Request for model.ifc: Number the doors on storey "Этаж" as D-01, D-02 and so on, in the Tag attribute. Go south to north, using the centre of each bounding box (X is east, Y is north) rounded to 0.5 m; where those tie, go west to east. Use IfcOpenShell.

First a look at what the model holds.

```python
import ifcopenshell
import ifcopenshell.util.element
import ifcopenshell.util.placement

model = ifcopenshell.open("model.ifc")
print(model.schema)
storey = next(s for s in model.by_type("IfcBuildingStorey") if s.Name == "Этаж")
doors = [e for e in ifcopenshell.util.element.get_decomposition(storey) if e.is_a("IfcDoor")]
for e in sorted(doors, key=lambda e: e.id()):
    origin = ifcopenshell.util.placement.get_local_placement(e.ObjectPlacement)[:3, 3]
    print(e.id(), e.Tag, e.Name, origin.round(2) + 0.0, sep=" | ")
```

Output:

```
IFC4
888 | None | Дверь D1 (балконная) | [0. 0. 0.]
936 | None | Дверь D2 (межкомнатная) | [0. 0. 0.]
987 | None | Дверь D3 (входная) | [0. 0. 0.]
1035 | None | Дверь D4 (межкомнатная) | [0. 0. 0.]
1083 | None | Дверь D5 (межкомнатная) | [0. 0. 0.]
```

```python
import ifcopenshell
import ifcopenshell.geom
import ifcopenshell.util.element
import ifcopenshell.util.shape

model = ifcopenshell.open("model.ifc")
settings = ifcopenshell.geom.settings()
settings.set("use-world-coords", True)


def centre(element):
    shape = ifcopenshell.geom.create_shape(settings, element)
    return ifcopenshell.util.shape.get_bbox_centroid(shape.geometry)


storey = next(s for s in model.by_type("IfcBuildingStorey") if s.Name == "Этаж")
doors = [e for e in ifcopenshell.util.element.get_decomposition(storey) if e.is_a("IfcDoor")]

# Insertion points can sit at a corner or the storey origin, so sort by the geometry (in metres).
centres = {e: centre(e) for e in doors}
doors.sort(key=lambda e: (round(centres[e][1] / 0.5), centres[e][0]))

for i, e in enumerate(doors, start=1):
    number = f"D-{i:02d}"
    e.Tag = number
    print(e.id(), number)

model.write("model_edited.ifc")
```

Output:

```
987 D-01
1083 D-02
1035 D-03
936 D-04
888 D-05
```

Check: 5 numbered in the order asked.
